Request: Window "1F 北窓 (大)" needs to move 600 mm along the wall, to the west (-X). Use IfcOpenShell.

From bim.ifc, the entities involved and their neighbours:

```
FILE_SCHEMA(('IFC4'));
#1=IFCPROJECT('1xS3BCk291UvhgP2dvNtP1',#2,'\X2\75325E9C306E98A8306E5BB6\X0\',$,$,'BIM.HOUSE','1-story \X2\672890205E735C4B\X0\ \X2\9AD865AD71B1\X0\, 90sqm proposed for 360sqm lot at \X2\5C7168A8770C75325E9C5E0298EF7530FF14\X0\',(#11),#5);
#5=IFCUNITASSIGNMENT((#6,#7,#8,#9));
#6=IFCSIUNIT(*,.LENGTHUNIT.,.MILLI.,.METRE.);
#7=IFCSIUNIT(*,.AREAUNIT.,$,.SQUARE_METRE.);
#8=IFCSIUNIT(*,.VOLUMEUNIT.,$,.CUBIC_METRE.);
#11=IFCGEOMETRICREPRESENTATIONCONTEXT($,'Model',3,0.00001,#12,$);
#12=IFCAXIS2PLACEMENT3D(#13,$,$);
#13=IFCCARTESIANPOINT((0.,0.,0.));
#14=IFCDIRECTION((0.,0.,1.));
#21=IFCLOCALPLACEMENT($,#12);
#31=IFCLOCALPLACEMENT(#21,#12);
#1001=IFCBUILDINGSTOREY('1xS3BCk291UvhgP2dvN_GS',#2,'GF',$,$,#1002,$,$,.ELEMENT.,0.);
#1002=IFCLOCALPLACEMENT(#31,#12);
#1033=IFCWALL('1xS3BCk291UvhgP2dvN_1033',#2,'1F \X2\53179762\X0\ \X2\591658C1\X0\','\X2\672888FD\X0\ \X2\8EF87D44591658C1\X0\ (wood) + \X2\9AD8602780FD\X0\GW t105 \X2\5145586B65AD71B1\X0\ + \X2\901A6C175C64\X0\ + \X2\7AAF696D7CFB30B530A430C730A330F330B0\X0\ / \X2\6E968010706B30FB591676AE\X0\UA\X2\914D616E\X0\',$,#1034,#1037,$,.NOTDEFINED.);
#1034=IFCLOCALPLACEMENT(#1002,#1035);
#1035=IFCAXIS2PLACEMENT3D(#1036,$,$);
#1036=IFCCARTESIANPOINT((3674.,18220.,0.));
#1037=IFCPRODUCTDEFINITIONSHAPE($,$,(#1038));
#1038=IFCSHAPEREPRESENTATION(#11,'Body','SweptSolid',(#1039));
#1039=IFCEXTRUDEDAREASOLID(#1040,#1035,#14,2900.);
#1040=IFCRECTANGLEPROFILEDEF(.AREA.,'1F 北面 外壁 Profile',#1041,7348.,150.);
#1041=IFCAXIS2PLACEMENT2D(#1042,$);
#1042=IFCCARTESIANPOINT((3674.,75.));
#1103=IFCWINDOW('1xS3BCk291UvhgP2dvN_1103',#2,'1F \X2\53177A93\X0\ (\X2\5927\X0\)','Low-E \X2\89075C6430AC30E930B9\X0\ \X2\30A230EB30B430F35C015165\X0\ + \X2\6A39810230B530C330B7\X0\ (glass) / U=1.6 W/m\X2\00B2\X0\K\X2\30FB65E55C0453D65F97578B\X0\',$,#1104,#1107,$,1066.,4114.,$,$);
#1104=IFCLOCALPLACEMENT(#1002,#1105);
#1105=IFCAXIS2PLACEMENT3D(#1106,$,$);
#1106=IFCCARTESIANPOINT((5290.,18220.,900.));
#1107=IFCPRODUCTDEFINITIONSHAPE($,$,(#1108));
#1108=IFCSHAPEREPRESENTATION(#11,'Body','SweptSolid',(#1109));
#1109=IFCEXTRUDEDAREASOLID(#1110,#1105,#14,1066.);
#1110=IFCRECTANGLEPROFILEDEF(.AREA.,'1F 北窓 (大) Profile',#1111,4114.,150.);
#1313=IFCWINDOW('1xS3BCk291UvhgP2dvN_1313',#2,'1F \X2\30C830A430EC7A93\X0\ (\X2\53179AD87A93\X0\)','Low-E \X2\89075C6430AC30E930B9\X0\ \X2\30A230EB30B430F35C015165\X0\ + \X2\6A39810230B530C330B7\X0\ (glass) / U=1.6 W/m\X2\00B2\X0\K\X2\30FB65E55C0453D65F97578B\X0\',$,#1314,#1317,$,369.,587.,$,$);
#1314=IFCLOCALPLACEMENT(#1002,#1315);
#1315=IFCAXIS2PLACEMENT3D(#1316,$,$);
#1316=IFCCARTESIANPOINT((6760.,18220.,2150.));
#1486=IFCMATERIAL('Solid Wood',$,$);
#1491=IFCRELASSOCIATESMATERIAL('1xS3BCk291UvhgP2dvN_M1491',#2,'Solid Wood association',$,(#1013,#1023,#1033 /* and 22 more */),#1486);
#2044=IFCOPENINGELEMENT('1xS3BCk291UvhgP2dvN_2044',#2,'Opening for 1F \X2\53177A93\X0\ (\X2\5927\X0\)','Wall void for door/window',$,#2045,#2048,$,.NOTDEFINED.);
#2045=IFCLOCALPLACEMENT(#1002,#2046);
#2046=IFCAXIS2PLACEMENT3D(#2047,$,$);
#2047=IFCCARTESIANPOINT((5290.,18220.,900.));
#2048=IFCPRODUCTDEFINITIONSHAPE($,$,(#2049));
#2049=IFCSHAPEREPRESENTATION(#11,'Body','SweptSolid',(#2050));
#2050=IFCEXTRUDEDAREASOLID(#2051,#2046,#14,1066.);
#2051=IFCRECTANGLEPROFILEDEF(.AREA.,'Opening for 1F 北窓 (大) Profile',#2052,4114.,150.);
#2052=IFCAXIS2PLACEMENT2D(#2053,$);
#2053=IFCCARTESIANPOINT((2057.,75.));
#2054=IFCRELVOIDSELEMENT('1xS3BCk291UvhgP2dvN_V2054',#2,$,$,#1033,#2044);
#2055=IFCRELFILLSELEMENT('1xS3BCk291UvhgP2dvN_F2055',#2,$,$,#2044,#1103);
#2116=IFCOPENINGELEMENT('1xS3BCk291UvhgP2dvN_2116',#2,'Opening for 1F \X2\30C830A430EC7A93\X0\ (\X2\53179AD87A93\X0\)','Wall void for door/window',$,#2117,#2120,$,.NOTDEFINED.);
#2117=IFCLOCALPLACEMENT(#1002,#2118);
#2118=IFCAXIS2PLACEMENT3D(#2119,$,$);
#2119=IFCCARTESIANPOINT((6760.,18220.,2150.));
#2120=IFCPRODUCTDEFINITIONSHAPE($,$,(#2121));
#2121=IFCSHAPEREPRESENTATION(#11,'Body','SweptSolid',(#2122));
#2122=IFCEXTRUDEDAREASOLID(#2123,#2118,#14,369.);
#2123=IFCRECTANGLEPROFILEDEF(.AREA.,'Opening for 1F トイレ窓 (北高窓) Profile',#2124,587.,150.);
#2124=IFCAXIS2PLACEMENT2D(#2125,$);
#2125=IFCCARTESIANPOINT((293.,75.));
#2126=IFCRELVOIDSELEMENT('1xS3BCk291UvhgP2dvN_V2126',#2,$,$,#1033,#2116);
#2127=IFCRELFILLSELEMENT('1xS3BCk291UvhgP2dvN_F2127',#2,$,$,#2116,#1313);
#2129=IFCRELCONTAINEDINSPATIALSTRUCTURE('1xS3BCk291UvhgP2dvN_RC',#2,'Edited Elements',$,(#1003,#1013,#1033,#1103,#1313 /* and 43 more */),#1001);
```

```python
import ifcopenshell
import ifcopenshell.api.geometry
import ifcopenshell.util.placement
import ifcopenshell.util.unit

model = ifcopenshell.open("bim.ifc")
unit_scale = ifcopenshell.util.unit.calculate_unit_scale(model)

window = model.by_guid("1xS3BCk291UvhgP2dvN_1103")
opening = window.FillsVoids[0].RelatingOpeningElement
wall = opening.VoidsElements[0].RelatingBuildingElement

wall_matrix = ifcopenshell.util.placement.get_local_placement(wall.ObjectPlacement)
shift = wall_matrix[:3, 0] * -0.6 / unit_scale
before = ifcopenshell.util.placement.get_local_placement(window.ObjectPlacement)[:3, 3].copy()

# The window is not placed relative to its opening, so move both.
for product in (opening, window):
    matrix = ifcopenshell.util.placement.get_local_placement(product.ObjectPlacement)
    matrix[:3, 3] += shift
    ifcopenshell.api.geometry.edit_object_placement(model, product=product, matrix=matrix, is_si=False)

after = ifcopenshell.util.placement.get_local_placement(window.ObjectPlacement)[:3, 3]
print("window moved by", (after - before).round(3) + 0.0)

model.write("bim_rev.ifc")
```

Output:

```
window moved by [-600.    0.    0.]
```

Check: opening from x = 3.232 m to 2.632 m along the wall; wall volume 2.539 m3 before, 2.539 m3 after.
